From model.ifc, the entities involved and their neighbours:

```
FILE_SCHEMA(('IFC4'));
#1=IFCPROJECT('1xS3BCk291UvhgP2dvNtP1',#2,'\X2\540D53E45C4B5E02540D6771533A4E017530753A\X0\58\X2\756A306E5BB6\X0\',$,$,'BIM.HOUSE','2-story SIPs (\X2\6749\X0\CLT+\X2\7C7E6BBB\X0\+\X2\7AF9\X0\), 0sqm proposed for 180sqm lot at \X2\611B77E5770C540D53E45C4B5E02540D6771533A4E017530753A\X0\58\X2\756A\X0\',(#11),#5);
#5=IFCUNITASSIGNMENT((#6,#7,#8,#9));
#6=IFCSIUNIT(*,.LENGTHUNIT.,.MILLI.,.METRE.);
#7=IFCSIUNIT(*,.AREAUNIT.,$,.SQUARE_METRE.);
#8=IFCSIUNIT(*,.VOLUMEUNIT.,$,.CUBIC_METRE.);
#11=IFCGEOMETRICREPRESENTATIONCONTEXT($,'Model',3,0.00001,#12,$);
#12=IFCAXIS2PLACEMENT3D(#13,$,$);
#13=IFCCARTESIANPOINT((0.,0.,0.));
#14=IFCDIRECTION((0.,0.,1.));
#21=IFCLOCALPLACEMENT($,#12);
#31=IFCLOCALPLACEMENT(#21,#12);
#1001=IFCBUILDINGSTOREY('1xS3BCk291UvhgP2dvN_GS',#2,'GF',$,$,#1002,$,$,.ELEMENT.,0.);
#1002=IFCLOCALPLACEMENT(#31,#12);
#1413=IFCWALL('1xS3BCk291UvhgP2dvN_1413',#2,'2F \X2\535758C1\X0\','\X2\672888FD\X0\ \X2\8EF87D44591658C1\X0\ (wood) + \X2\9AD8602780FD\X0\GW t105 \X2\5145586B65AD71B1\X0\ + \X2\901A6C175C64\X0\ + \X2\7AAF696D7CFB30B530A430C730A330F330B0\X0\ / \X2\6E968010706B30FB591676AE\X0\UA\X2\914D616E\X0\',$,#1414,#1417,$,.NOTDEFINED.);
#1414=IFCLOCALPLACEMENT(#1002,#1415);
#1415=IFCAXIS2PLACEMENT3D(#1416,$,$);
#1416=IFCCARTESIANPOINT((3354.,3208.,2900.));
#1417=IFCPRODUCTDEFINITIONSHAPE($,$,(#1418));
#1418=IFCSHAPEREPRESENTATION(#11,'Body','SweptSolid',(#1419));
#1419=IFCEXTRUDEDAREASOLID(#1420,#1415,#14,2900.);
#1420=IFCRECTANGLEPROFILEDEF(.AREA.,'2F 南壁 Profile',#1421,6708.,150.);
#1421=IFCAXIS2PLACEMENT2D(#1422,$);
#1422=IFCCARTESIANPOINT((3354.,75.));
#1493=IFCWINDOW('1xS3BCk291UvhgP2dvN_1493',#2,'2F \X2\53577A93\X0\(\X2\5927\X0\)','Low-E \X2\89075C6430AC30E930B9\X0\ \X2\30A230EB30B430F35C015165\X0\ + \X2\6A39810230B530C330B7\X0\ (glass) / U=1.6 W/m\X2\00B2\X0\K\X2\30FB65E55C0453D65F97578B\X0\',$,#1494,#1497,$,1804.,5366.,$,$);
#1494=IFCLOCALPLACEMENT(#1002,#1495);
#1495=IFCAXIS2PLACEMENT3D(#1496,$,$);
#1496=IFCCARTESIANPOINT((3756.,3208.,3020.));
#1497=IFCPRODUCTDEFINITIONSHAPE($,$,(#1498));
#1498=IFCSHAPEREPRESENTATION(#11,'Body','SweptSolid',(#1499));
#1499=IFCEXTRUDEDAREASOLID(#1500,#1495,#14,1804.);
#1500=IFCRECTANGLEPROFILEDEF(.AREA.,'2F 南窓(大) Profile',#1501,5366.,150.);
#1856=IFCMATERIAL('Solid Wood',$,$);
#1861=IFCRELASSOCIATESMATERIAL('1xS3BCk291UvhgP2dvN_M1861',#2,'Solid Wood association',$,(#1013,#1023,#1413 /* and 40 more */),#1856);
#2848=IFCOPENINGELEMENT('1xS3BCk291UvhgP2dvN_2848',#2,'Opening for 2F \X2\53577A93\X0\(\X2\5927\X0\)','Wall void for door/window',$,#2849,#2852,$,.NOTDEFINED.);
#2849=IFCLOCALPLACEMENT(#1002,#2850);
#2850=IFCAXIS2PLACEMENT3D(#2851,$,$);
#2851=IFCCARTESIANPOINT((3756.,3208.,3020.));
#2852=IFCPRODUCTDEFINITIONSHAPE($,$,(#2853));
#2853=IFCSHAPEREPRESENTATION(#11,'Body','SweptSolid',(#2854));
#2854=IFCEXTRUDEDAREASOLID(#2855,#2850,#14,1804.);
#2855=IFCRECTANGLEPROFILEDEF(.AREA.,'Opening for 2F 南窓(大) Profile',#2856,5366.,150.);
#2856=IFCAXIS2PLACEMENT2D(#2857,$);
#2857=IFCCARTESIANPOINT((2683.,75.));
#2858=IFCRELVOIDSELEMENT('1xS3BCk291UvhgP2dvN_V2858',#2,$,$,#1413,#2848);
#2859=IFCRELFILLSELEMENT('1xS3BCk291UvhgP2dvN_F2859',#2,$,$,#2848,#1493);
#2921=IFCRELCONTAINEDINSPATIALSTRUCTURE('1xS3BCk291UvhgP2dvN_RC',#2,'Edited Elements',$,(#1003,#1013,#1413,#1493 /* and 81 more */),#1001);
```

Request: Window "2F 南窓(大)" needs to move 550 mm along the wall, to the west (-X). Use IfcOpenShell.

```python
import ifcopenshell
import ifcopenshell.api.geometry
import ifcopenshell.util.placement
import ifcopenshell.util.unit

model = ifcopenshell.open("model.ifc")
unit_scale = ifcopenshell.util.unit.calculate_unit_scale(model)

window = model.by_guid("1xS3BCk291UvhgP2dvN_1493")
opening = window.FillsVoids[0].RelatingOpeningElement
wall = opening.VoidsElements[0].RelatingBuildingElement

wall_matrix = ifcopenshell.util.placement.get_local_placement(wall.ObjectPlacement)
shift = wall_matrix[:3, 0] * -0.55 / unit_scale
before = ifcopenshell.util.placement.get_local_placement(window.ObjectPlacement)[:3, 3].copy()

# The window is not placed relative to its opening, so move both.
for product in (opening, window):
    matrix = ifcopenshell.util.placement.get_local_placement(product.ObjectPlacement)
    matrix[:3, 3] += shift
    ifcopenshell.api.geometry.edit_object_placement(model, product=product, matrix=matrix, is_si=False)

after = ifcopenshell.util.placement.get_local_placement(window.ObjectPlacement)[:3, 3]
print("window moved by", (after - before).round(3) + 0.0)

model.write("model_updated.ifc")
```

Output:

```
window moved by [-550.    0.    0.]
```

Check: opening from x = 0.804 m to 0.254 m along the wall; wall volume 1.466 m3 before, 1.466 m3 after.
